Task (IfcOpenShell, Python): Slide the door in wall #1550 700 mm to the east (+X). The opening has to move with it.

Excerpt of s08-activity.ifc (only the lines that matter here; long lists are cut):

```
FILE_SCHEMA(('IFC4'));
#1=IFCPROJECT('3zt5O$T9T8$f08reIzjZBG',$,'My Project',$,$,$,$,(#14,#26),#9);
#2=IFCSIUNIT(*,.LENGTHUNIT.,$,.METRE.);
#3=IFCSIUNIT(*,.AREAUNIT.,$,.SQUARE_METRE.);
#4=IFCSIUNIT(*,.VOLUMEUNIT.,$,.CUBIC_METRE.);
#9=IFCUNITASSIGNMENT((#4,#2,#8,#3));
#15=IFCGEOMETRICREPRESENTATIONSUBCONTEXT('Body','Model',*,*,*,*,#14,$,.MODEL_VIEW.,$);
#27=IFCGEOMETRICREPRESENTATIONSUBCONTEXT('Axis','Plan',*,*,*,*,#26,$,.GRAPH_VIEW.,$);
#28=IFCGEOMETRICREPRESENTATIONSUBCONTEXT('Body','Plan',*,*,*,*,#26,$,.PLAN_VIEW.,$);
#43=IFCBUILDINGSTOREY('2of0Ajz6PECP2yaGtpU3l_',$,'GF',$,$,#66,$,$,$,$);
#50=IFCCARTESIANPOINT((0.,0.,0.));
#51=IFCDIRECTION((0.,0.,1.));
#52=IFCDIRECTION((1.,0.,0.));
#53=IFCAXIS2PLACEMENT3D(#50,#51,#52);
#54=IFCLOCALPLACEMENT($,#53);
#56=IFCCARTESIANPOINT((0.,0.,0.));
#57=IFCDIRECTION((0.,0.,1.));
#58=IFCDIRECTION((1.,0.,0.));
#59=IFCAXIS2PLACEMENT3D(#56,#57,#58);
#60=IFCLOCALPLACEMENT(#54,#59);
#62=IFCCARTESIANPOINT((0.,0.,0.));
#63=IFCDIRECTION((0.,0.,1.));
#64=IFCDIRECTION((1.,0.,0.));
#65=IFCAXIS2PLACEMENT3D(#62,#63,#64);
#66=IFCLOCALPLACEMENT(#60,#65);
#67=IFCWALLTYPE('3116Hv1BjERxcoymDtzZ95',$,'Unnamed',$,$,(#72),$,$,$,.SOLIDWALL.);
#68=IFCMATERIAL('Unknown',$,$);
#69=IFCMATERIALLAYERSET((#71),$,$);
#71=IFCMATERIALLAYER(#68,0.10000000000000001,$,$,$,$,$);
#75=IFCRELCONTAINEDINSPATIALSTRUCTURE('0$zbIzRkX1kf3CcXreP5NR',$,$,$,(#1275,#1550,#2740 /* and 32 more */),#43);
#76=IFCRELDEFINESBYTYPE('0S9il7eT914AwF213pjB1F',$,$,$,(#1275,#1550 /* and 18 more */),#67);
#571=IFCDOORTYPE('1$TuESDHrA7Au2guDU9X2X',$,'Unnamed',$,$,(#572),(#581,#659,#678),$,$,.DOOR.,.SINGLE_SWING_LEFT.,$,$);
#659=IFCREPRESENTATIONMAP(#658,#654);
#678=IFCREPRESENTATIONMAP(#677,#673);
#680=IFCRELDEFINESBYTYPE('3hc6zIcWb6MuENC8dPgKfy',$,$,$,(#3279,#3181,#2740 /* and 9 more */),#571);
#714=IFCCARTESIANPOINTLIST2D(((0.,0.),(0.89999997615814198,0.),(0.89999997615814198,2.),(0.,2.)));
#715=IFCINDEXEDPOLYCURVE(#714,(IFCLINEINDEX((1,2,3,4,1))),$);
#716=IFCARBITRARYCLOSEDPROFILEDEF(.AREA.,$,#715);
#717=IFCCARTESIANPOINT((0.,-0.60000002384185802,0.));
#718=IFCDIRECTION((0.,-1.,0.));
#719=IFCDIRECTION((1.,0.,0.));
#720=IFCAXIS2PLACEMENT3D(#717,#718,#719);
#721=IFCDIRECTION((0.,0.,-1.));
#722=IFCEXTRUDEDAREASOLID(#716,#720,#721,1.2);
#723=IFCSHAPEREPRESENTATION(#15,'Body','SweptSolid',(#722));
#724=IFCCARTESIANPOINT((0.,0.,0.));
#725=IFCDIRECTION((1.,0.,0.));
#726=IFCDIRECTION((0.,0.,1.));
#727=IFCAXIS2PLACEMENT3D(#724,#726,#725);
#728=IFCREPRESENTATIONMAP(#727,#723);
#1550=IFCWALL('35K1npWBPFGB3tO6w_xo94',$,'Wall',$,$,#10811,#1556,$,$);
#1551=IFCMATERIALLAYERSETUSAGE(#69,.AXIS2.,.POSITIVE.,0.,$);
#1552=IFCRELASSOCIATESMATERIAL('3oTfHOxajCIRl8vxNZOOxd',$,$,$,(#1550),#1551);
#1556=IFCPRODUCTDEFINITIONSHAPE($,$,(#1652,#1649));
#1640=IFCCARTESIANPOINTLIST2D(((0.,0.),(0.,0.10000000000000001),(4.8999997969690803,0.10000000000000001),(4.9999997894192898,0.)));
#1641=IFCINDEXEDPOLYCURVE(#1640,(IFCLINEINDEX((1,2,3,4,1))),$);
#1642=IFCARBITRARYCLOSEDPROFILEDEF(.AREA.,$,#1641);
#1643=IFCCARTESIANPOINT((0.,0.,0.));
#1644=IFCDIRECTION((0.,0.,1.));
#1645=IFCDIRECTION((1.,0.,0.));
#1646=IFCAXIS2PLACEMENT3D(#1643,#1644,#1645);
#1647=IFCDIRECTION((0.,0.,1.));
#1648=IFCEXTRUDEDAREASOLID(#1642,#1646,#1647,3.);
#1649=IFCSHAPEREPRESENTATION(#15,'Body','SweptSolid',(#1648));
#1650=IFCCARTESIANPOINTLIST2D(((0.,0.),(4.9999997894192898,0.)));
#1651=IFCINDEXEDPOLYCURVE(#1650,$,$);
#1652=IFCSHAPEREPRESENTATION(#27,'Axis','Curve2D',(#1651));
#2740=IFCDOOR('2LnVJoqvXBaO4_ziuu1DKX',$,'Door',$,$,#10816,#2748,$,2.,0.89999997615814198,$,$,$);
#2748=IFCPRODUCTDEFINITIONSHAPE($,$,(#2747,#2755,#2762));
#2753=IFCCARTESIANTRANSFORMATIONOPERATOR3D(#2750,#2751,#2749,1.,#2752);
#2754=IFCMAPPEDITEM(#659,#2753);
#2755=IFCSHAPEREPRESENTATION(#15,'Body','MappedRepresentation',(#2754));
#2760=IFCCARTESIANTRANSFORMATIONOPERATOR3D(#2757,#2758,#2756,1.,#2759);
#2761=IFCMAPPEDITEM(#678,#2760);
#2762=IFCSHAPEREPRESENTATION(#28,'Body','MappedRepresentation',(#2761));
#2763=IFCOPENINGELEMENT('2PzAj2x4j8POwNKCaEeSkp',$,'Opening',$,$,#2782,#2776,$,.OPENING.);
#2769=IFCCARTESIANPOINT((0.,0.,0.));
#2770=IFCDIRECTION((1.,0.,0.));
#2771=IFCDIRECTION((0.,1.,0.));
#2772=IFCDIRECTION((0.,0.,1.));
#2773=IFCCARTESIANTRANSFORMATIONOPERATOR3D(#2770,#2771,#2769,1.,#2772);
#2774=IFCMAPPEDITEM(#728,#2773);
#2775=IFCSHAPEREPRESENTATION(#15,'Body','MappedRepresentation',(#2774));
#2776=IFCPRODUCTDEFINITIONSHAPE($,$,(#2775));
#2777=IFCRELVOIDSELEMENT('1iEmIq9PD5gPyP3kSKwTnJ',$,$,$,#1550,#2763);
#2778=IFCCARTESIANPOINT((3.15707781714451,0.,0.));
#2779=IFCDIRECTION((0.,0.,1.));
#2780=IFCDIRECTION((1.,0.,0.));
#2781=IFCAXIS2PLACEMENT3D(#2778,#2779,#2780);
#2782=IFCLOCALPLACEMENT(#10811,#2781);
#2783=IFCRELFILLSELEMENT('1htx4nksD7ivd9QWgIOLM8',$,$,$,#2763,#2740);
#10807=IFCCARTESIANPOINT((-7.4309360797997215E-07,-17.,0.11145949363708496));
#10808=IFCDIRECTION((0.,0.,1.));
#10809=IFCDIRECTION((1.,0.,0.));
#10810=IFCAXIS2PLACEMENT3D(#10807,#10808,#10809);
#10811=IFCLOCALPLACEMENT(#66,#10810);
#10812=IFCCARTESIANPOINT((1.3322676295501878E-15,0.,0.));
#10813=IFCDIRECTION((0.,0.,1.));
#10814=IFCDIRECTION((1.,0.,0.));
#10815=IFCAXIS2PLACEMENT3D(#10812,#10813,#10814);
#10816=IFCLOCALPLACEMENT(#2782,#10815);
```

```python
import ifcopenshell
import ifcopenshell.api.geometry
import ifcopenshell.util.placement
import ifcopenshell.util.unit

model = ifcopenshell.open("s08-activity.ifc")
unit_scale = ifcopenshell.util.unit.calculate_unit_scale(model)

door = model.by_guid("2LnVJoqvXBaO4_ziuu1DKX")
opening = door.FillsVoids[0].RelatingOpeningElement
wall = opening.VoidsElements[0].RelatingBuildingElement

wall_matrix = ifcopenshell.util.placement.get_local_placement(wall.ObjectPlacement)
shift = wall_matrix[:3, 0] * 0.7 / unit_scale
before = ifcopenshell.util.placement.get_local_placement(door.ObjectPlacement)[:3, 3].copy()

# The door is placed relative to its opening, so it follows when the opening moves.
matrix = ifcopenshell.util.placement.get_local_placement(opening.ObjectPlacement)
matrix[:3, 3] += shift
ifcopenshell.api.geometry.edit_object_placement(
    model, product=opening, matrix=matrix, is_si=False, should_transform_children=True
)

after = ifcopenshell.util.placement.get_local_placement(door.ObjectPlacement)[:3, 3]
print("door moved by", (after - before).round(3) + 0.0)

model.write("s08-activity_edited.ifc")
```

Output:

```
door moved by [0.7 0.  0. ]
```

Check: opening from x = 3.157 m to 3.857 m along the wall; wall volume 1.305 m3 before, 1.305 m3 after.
